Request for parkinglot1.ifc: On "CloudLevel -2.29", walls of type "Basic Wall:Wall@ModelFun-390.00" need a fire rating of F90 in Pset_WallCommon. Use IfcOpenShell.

First a look at what the model holds.

```python
import ifcopenshell
import ifcopenshell.util.element

model = ifcopenshell.open("parkinglot1.ifc")
print(model.schema)
storey = next(s for s in model.by_type("IfcBuildingStorey") if s.Name == "CloudLevel -2.29")
walls = [e for e in ifcopenshell.util.element.get_decomposition(storey) if e.is_a("IfcWall")]
seen = {}
for e in walls:
    element_type = ifcopenshell.util.element.get_type(e)
    key = (element_type.Name if element_type != e and element_type else None, ifcopenshell.util.element.get_pset(e, "Pset_WallCommon", "FireRating"))
    seen[key] = seen.get(key, 0) + 1
for (name, value), count in sorted(seen.items(), key=str):
    print(count, "x", name, "|", value)
```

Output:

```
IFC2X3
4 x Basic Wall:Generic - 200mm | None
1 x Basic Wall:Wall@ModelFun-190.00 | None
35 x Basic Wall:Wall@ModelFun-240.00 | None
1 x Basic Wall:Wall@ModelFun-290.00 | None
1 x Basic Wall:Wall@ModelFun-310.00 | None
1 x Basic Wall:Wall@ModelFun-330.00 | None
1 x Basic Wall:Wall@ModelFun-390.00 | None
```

```python
import ifcopenshell
import ifcopenshell.api.pset
import ifcopenshell.util.element

model = ifcopenshell.open("parkinglot1.ifc")

storey = next(s for s in model.by_type("IfcBuildingStorey") if s.Name == "CloudLevel -2.29")
walls = [e for e in ifcopenshell.util.element.get_decomposition(storey) if e.is_a("IfcWall")]

count = 0
for e in walls:
    element_type = ifcopenshell.util.element.get_type(e)
    if element_type in (None, e) or element_type.Name != "Basic Wall:Wall@ModelFun-390.00":
        continue
    # add_pset returns the element's existing set when there is one.
    pset = ifcopenshell.api.pset.add_pset(model, product=e, name="Pset_WallCommon")
    ifcopenshell.api.pset.edit_pset(model, pset=pset, properties={"FireRating": "F90"})
    count += 1

print(count, "walls updated")

model.write("parkinglot1-out.ifc")
```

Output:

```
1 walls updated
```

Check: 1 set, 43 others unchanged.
